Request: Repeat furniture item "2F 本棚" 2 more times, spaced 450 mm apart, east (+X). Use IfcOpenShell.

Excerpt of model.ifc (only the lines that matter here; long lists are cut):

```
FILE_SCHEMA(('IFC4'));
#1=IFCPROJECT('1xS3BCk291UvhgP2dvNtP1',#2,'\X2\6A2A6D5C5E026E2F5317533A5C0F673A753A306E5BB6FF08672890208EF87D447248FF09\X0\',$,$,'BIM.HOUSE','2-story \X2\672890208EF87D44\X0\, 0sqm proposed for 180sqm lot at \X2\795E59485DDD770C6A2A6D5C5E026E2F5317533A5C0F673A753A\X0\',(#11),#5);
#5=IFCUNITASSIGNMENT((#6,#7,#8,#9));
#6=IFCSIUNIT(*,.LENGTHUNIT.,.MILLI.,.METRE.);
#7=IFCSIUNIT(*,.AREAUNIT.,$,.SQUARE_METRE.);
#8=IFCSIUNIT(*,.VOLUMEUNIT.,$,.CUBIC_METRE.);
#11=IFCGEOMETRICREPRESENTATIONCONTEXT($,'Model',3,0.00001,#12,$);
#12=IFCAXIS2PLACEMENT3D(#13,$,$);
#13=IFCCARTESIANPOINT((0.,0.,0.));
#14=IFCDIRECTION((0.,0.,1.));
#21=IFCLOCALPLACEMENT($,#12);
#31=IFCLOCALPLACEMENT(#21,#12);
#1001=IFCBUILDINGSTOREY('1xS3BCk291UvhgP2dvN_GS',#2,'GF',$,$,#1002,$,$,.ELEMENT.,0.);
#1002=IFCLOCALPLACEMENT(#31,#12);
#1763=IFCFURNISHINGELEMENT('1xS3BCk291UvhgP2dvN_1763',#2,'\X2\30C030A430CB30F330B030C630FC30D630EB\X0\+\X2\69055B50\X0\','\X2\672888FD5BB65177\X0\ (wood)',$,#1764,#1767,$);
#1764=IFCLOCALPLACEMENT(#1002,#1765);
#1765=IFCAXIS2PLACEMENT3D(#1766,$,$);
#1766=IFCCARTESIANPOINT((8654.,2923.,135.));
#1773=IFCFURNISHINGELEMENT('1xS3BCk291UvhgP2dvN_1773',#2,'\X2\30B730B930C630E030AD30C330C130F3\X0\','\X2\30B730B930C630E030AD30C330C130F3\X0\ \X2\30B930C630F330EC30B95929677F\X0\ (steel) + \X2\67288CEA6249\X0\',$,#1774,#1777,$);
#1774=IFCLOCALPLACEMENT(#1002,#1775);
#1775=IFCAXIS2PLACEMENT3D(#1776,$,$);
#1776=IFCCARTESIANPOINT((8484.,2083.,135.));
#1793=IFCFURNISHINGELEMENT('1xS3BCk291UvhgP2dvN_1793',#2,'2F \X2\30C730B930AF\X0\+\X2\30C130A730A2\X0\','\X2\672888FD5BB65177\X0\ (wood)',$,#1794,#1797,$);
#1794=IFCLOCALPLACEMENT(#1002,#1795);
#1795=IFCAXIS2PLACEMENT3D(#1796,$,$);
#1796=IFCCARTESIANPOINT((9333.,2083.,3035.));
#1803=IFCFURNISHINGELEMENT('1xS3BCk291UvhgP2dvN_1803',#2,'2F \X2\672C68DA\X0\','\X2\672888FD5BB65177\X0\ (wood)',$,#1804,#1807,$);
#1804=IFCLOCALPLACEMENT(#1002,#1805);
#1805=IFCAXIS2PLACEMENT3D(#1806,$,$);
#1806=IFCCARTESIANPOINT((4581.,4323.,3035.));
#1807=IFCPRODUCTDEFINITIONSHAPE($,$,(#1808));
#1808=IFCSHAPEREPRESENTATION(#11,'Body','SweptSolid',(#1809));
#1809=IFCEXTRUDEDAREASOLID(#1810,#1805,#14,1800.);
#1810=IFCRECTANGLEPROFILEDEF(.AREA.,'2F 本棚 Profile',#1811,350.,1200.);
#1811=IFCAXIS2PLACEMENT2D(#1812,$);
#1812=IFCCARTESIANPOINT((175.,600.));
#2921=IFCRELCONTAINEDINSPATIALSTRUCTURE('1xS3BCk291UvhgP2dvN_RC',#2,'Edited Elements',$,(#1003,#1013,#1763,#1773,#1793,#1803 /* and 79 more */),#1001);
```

```python
import numpy as np
import ifcopenshell
import ifcopenshell.api.geometry
import ifcopenshell.api.root
import ifcopenshell.util.element
import ifcopenshell.util.placement

model = ifcopenshell.open("model.ifc")


def reuse_history(source, copy):
    """copy_class also copies each property set's owner history, people and application; keep the originals."""
    for rel in copy.IsDefinedBy:
        if rel.is_a("IfcRelDefinesByProperties") and (history := rel.RelatingPropertyDefinition.OwnerHistory):
            rel.RelatingPropertyDefinition.OwnerHistory = source.OwnerHistory
            ifcopenshell.util.element.remove_deep2(model, history)


source = model.by_guid("1xS3BCk291UvhgP2dvN_1803")
base = ifcopenshell.util.placement.get_local_placement(source.ObjectPlacement)
step = np.array([1.0, 0.0, 0.0]) * 450.0

for i in range(1, 3):
    copy = ifcopenshell.api.root.copy_class(model, product=source)
    copy.Representation = ifcopenshell.util.element.copy_deep(
        model, source.Representation, exclude=["IfcGeometricRepresentationContext", "IfcRepresentationMap"]
    )
    reuse_history(source, copy)
    matrix = base.copy()
    matrix[:3, 3] += i * step
    print("added at", matrix[:3, 3].round(3) + 0.0)
    ifcopenshell.api.geometry.edit_object_placement(model, product=copy, matrix=matrix, is_si=False)

model.write("model-out.ifc")
```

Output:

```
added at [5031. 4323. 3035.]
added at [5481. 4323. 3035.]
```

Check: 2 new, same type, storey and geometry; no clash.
